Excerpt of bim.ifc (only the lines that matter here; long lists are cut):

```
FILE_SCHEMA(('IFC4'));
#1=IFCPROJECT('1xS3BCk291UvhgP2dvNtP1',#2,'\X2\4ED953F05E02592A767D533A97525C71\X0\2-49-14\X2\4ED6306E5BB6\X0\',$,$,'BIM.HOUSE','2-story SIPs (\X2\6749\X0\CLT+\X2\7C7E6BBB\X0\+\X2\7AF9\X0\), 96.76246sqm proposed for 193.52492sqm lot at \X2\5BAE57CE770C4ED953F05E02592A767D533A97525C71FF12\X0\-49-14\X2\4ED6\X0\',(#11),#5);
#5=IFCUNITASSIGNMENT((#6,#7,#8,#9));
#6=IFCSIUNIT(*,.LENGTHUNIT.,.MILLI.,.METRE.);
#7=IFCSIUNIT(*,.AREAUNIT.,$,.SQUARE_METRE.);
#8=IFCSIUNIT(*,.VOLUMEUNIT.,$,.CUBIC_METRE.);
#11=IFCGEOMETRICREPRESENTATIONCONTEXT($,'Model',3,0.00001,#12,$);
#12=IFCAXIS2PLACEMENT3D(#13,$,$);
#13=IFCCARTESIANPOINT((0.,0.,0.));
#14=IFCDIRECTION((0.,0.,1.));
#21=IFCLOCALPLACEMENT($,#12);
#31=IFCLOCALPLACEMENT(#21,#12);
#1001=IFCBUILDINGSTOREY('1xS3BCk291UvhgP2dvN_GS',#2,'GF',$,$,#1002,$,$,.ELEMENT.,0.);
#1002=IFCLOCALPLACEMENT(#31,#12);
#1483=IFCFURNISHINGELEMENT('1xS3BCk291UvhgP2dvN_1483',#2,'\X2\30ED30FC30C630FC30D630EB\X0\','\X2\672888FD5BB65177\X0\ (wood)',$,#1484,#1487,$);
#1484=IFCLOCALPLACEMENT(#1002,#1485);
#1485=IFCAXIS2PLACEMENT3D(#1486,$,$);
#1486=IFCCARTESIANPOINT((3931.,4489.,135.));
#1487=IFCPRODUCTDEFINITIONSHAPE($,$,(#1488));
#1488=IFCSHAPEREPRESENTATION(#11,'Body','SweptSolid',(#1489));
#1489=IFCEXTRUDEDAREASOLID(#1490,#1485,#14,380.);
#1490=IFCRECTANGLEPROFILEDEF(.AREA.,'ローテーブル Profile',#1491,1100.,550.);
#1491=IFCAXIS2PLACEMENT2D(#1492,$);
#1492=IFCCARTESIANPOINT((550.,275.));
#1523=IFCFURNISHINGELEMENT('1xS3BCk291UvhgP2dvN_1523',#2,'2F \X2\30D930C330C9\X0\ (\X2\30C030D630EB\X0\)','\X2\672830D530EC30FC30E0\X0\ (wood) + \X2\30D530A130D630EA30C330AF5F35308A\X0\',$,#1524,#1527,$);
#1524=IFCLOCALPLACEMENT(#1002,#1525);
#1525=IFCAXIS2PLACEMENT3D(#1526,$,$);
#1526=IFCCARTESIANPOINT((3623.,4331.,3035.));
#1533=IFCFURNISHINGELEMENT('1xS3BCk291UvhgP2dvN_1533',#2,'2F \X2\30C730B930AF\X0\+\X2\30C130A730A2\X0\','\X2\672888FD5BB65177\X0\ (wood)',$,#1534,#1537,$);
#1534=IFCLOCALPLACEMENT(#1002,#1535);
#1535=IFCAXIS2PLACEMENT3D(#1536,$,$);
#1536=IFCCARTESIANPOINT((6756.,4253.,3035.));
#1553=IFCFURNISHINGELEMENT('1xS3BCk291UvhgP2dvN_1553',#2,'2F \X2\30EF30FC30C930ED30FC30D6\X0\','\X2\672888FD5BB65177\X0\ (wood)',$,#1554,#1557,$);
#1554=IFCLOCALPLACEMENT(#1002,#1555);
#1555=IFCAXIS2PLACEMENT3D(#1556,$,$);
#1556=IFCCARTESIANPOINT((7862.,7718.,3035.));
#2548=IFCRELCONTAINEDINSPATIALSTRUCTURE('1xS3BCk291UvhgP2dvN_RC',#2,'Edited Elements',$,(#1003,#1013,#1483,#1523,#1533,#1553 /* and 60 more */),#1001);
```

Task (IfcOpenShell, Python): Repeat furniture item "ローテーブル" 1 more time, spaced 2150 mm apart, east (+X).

```python
import numpy as np
import ifcopenshell
import ifcopenshell.api.geometry
import ifcopenshell.api.root
import ifcopenshell.util.element
import ifcopenshell.util.placement
import ifcopenshell.util.unit

model = ifcopenshell.open("bim.ifc")
unit_scale = ifcopenshell.util.unit.calculate_unit_scale(model)


def reuse_history(source, copy):
    """copy_class also copies each property set's owner history, people and application; keep the originals."""
    for rel in copy.IsDefinedBy:
        if rel.is_a("IfcRelDefinesByProperties") and (history := rel.RelatingPropertyDefinition.OwnerHistory):
            rel.RelatingPropertyDefinition.OwnerHistory = source.OwnerHistory
            ifcopenshell.util.element.remove_deep2(model, history)


source = model.by_guid("1xS3BCk291UvhgP2dvN_1483")
base = ifcopenshell.util.placement.get_local_placement(source.ObjectPlacement)
step = np.array([1.0, 0.0, 0.0]) * 2.15 / unit_scale

for i in range(1, 2):
    copy = ifcopenshell.api.root.copy_class(model, product=source)
    copy.Representation = ifcopenshell.util.element.copy_deep(
        model, source.Representation, exclude=["IfcGeometricRepresentationContext", "IfcRepresentationMap"]
    )
    reuse_history(source, copy)
    matrix = base.copy()
    matrix[:3, 3] += i * step
    print("added at", matrix[:3, 3].round(3) + 0.0)
    ifcopenshell.api.geometry.edit_object_placement(model, product=copy, matrix=matrix, is_si=False)

model.write("bim_edited.ifc")
```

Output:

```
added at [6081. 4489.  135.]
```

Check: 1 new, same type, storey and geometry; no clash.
